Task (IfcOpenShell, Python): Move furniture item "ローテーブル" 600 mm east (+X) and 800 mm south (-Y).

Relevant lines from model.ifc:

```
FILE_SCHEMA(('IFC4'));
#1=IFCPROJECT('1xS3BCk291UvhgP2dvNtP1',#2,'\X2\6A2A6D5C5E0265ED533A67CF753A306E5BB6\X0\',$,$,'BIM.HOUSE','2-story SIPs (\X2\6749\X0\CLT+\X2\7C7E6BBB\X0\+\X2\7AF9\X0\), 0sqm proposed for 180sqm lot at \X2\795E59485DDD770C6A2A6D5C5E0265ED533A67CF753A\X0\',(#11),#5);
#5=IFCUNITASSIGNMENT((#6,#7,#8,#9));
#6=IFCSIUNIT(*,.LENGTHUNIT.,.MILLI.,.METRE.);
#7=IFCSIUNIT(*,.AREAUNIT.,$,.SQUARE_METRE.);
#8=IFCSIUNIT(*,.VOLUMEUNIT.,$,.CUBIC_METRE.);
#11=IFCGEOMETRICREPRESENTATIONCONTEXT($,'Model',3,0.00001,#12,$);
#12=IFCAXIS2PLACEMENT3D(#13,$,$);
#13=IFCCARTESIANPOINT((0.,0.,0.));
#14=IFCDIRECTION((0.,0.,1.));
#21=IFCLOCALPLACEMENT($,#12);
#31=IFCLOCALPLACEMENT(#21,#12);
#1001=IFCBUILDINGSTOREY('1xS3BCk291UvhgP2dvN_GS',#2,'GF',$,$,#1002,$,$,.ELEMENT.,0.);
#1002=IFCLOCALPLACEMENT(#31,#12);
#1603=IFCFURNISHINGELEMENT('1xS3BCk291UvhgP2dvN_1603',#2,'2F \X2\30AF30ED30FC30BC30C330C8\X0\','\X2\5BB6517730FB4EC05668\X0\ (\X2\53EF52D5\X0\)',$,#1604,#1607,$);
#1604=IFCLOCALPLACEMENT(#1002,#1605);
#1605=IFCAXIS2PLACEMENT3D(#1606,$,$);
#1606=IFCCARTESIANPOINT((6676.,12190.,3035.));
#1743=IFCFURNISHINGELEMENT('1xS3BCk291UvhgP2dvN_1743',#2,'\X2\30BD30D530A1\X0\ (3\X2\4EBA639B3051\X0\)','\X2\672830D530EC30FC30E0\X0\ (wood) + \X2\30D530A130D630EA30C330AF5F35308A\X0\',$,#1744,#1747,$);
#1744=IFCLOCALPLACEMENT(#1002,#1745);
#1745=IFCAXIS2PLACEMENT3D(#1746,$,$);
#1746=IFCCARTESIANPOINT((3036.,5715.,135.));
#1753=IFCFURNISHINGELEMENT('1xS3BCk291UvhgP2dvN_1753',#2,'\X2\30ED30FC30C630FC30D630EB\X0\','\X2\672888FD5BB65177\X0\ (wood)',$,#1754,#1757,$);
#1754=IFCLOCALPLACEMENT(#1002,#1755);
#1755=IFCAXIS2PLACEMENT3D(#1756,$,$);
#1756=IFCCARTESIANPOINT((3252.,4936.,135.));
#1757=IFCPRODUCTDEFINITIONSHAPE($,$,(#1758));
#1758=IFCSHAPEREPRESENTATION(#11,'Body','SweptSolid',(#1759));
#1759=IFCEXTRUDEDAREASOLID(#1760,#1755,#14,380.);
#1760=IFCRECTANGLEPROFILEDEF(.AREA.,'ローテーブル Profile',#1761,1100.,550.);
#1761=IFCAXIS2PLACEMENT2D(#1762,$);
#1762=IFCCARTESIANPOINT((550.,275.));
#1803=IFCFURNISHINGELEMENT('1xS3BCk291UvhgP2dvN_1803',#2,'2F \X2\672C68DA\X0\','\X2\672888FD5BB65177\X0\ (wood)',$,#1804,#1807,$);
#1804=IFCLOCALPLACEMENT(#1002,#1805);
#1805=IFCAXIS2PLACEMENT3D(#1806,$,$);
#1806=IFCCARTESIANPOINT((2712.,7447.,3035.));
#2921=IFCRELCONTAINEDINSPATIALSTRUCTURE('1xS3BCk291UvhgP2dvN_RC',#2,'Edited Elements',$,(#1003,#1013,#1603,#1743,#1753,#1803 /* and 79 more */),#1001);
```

```python
import ifcopenshell
import ifcopenshell.api.geometry
import ifcopenshell.util.placement

model = ifcopenshell.open("model.ifc")

item = model.by_guid("1xS3BCk291UvhgP2dvN_1753")
matrix = ifcopenshell.util.placement.get_local_placement(item.ObjectPlacement)
matrix[0, 3] += 600.0
matrix[1, 3] -= 800.0
ifcopenshell.api.geometry.edit_object_placement(model, product=item, matrix=matrix, is_si=False)

print(ifcopenshell.util.placement.get_local_placement(item.ObjectPlacement).round(3) + 0.0)

model.write("model_v2.ifc")
```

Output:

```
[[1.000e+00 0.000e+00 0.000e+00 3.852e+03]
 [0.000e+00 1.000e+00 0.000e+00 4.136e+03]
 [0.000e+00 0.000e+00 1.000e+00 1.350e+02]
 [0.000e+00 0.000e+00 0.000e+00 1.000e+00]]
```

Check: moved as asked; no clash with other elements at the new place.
